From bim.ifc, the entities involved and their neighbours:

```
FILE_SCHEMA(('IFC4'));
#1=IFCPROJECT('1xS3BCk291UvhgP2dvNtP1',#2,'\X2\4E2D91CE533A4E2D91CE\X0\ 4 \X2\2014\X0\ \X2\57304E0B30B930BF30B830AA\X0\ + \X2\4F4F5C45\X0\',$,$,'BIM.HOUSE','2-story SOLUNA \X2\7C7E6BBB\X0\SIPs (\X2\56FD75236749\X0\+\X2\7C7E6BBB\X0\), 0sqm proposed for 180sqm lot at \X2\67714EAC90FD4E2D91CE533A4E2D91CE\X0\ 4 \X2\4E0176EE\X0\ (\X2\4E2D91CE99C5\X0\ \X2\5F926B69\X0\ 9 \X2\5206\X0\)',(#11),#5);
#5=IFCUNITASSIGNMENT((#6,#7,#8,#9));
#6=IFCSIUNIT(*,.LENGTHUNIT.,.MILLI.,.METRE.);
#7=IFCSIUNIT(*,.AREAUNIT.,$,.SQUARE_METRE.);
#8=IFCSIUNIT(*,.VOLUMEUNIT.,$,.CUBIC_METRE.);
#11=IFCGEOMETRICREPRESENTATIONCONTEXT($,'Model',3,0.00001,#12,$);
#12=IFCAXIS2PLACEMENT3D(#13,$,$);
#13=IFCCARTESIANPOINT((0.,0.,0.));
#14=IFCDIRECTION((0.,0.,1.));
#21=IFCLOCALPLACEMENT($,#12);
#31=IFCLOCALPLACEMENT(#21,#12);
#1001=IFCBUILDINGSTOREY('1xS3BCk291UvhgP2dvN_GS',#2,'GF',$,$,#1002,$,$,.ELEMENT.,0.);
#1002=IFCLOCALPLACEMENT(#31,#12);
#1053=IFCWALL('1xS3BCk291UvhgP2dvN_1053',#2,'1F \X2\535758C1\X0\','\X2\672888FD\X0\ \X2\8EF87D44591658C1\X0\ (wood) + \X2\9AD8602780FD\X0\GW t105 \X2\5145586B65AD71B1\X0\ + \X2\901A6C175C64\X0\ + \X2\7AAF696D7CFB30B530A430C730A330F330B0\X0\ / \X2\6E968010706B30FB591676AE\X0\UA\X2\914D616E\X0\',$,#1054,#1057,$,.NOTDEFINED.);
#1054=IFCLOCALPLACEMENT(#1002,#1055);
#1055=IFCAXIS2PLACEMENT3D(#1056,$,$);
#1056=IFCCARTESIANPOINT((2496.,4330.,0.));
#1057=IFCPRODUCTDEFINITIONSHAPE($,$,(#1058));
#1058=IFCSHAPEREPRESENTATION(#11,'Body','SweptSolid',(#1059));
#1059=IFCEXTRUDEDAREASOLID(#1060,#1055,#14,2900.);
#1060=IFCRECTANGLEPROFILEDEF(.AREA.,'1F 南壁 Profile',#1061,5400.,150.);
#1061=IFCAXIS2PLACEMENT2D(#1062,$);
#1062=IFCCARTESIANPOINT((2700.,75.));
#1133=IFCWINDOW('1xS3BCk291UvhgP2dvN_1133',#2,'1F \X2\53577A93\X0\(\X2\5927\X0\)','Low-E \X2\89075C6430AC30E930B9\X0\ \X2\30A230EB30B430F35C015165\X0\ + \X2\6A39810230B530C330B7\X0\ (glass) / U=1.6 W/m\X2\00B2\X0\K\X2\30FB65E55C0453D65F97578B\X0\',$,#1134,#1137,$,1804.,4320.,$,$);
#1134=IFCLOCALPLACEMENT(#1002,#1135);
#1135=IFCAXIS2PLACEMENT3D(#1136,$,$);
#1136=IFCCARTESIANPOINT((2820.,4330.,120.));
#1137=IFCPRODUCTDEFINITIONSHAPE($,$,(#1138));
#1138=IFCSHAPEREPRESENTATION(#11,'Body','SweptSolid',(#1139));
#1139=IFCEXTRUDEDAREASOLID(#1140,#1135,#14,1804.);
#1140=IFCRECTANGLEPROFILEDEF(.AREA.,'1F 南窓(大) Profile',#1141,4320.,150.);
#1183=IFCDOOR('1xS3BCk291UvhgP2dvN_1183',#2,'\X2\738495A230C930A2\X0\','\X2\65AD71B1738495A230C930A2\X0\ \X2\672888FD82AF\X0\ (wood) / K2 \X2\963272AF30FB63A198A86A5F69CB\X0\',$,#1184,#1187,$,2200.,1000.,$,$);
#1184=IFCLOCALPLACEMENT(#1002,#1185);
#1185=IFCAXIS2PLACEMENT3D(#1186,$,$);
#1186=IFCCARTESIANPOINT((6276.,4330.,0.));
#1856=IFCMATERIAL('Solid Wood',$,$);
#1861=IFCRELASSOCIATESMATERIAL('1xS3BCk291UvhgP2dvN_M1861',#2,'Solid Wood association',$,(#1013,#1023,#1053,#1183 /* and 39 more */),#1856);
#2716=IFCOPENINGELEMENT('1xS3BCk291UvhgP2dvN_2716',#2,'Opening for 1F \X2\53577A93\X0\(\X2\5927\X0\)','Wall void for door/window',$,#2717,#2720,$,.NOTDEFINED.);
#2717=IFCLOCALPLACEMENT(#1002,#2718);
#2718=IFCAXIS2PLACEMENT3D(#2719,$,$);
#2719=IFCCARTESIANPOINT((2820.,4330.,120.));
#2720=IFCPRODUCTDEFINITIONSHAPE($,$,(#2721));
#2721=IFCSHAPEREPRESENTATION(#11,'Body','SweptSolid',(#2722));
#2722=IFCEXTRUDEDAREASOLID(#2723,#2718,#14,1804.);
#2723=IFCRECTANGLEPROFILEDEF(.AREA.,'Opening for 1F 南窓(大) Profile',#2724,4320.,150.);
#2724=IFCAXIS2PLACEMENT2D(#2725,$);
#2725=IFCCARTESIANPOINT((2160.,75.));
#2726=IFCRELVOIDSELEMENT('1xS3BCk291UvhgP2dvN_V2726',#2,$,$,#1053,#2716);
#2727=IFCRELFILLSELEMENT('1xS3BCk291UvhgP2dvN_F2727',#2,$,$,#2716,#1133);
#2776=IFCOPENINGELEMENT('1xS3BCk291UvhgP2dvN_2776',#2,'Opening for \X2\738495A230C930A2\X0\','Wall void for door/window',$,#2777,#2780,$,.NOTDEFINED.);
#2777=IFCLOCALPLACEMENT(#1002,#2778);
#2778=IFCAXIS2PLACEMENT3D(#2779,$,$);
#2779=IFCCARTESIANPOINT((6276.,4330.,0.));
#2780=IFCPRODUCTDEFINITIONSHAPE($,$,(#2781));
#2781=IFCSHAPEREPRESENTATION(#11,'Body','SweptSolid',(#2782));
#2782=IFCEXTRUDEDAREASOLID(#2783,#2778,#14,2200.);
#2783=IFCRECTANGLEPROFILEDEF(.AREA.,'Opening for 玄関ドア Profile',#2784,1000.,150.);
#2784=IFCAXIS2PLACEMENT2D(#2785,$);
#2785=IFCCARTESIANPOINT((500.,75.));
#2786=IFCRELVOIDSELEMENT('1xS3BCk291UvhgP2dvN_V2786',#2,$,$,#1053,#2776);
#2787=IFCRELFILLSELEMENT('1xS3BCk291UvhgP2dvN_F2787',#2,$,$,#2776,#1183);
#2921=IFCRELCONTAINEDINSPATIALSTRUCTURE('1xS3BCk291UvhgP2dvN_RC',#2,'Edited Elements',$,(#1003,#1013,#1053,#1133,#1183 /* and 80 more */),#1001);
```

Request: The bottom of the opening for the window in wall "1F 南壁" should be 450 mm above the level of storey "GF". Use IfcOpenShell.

```python
import numpy as np
import ifcopenshell
import ifcopenshell.api.geometry
import ifcopenshell.geom
import ifcopenshell.util.element
import ifcopenshell.util.placement
import ifcopenshell.util.shape
import ifcopenshell.util.unit

model = ifcopenshell.open("bim.ifc")
unit_scale = ifcopenshell.util.unit.calculate_unit_scale(model)

window = model.by_guid("1xS3BCk291UvhgP2dvN_1133")
opening = window.FillsVoids[0].RelatingOpeningElement
storey = ifcopenshell.util.element.get_container(window, ifc_class="IfcBuildingStorey")
level = ifcopenshell.util.placement.get_local_placement(storey.ObjectPlacement)[2, 3]

# The opening's origin need not be at the sill, so measure its lowest point.
shape = ifcopenshell.geom.create_shape(ifcopenshell.geom.settings(), opening)
bottom = ifcopenshell.util.shape.get_shape_bottom_elevation(shape, shape.geometry) / unit_scale
dz = level + 0.45 / unit_scale - bottom

shift = np.array([0.0, 0.0, dz])
# The window is not placed relative to its opening, so move both.
for product in (opening, window):
    matrix = ifcopenshell.util.placement.get_local_placement(product.ObjectPlacement)
    matrix[:3, 3] += shift
    ifcopenshell.api.geometry.edit_object_placement(model, product=product, matrix=matrix, is_si=False)

print(f"moved by {dz * unit_scale:+.3f} m")

model.write("bim-out.ifc")
```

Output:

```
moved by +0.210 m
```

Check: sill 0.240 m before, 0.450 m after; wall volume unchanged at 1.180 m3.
